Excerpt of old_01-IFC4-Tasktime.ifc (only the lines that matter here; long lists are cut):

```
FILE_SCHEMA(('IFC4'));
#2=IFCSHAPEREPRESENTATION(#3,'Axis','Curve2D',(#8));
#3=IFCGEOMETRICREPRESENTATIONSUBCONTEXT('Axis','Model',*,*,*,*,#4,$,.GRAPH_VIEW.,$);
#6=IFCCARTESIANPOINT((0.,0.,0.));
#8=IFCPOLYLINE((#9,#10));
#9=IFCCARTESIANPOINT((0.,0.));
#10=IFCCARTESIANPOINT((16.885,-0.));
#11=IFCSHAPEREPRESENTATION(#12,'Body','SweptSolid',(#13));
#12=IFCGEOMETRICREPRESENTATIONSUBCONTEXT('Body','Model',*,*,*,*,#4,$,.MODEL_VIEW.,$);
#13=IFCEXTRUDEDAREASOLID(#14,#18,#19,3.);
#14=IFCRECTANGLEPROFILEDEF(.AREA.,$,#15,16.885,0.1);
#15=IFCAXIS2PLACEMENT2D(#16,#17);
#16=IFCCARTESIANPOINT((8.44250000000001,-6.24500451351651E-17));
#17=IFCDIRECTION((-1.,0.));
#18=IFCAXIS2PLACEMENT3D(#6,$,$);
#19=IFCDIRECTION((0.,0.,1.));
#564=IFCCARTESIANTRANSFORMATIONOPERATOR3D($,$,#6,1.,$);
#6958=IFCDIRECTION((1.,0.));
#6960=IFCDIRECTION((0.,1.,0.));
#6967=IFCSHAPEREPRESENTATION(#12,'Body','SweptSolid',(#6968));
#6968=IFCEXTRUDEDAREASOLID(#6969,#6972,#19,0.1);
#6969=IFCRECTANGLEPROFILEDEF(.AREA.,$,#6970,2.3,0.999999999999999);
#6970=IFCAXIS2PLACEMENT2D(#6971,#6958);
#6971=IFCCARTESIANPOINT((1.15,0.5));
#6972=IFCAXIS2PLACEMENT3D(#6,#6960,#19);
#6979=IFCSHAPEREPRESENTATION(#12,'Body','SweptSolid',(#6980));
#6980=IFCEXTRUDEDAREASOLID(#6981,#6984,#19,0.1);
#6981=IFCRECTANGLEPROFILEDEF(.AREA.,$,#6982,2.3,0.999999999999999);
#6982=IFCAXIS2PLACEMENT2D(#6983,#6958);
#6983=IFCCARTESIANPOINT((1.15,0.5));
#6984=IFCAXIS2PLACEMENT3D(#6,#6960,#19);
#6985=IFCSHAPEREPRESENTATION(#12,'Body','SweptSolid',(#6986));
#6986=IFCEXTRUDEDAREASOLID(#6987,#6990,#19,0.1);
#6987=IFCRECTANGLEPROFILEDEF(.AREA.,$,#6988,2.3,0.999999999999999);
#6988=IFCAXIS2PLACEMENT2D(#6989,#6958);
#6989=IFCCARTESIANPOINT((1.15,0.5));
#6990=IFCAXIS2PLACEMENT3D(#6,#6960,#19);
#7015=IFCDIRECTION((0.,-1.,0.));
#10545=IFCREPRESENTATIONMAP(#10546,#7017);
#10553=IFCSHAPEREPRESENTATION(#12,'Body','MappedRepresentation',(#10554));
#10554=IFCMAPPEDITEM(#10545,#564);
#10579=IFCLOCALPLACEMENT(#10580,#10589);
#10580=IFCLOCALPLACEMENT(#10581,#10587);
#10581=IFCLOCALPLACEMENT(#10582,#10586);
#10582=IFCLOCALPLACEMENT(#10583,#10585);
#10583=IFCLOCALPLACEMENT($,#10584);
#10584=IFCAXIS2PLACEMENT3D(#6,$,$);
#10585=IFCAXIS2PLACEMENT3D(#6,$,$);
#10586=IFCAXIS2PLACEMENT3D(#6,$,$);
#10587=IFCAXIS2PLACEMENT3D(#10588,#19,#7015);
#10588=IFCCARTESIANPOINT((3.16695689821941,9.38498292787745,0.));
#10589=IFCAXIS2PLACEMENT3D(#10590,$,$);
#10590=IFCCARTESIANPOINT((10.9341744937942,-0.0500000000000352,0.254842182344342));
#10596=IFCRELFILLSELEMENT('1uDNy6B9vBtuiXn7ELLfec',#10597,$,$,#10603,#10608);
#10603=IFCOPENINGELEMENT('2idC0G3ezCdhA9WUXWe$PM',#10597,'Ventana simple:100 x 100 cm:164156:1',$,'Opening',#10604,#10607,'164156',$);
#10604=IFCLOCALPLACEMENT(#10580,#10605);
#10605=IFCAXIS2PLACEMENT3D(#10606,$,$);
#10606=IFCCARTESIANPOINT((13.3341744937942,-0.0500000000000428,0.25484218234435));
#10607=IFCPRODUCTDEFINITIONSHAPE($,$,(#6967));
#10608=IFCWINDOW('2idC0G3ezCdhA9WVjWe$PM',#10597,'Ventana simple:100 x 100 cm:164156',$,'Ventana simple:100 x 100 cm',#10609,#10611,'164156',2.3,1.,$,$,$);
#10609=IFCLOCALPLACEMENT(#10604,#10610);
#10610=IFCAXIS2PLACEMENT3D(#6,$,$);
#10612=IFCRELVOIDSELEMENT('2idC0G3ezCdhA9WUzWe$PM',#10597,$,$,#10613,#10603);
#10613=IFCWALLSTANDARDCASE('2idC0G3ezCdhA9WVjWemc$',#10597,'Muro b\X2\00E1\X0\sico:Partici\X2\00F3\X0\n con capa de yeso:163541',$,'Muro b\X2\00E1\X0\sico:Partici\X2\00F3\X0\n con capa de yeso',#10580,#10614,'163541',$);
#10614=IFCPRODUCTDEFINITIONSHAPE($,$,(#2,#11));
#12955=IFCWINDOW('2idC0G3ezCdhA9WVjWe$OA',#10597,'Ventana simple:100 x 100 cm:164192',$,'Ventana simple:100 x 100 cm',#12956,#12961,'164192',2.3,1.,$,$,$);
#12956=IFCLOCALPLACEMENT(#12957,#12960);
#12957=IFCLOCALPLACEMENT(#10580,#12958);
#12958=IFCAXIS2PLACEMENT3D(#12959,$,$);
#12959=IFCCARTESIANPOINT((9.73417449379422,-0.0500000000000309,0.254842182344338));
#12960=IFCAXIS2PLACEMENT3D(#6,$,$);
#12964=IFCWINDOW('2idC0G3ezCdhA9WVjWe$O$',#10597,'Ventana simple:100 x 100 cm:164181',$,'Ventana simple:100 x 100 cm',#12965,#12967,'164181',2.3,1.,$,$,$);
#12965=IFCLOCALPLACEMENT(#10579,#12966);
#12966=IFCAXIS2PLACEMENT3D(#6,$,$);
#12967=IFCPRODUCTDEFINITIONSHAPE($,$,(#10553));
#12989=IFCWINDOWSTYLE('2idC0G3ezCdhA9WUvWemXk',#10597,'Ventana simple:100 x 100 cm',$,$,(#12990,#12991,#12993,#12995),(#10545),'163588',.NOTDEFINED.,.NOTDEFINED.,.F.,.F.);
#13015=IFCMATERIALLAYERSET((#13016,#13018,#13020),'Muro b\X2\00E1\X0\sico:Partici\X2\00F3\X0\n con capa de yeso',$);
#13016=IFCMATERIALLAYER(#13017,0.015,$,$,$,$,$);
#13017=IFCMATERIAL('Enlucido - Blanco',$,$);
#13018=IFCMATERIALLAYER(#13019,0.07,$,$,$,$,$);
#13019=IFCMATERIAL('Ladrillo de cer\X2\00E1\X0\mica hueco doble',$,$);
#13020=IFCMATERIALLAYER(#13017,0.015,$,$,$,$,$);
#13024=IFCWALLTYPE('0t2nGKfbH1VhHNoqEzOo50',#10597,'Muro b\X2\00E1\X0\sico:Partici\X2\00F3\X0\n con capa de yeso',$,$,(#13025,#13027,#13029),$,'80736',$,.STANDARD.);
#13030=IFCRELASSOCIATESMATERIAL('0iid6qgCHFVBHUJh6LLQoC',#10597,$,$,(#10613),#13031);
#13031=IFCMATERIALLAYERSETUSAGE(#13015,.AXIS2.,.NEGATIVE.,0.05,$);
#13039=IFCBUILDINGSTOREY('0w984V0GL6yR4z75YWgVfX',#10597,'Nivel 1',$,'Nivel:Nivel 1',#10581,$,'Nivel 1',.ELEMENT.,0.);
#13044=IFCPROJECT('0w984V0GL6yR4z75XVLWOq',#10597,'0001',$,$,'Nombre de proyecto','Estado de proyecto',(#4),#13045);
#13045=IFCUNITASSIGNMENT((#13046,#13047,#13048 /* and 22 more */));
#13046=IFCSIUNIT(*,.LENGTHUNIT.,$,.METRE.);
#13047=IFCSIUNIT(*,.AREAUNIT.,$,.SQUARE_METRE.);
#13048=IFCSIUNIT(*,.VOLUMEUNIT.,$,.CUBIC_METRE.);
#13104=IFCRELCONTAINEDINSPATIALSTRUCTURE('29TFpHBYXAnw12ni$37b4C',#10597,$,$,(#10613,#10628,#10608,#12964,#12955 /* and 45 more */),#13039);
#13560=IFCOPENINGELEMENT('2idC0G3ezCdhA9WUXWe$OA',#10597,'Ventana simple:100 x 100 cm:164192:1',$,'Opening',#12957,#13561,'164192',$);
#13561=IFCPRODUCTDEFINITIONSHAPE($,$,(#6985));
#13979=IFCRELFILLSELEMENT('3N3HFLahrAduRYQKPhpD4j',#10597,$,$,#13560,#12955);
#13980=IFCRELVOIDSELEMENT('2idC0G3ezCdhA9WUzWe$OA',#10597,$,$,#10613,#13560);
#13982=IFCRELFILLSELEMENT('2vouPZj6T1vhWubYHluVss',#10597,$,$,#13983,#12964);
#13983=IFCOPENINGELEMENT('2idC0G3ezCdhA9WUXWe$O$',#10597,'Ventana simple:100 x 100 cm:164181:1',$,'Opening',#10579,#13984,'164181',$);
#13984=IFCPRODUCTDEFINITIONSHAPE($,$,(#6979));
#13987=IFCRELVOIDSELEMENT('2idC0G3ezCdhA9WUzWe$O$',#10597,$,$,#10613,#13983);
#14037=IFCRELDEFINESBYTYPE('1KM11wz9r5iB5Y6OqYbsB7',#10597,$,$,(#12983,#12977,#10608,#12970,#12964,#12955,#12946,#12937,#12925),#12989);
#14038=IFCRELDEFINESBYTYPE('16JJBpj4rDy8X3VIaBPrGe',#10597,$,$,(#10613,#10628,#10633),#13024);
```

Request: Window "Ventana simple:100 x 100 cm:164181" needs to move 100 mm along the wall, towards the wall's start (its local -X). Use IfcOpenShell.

```python
import ifcopenshell
import ifcopenshell.api.geometry
import ifcopenshell.util.placement

model = ifcopenshell.open("old_01-IFC4-Tasktime.ifc")

window = model.by_guid("2idC0G3ezCdhA9WVjWe$O$")
opening = window.FillsVoids[0].RelatingOpeningElement
wall = opening.VoidsElements[0].RelatingBuildingElement

wall_matrix = ifcopenshell.util.placement.get_local_placement(wall.ObjectPlacement)
shift = wall_matrix[:3, 0] * -0.1
before = ifcopenshell.util.placement.get_local_placement(window.ObjectPlacement)[:3, 3].copy()

# The window is placed relative to its opening, so it follows when the opening moves.
matrix = ifcopenshell.util.placement.get_local_placement(opening.ObjectPlacement)
matrix[:3, 3] += shift
ifcopenshell.api.geometry.edit_object_placement(
    model, product=opening, matrix=matrix, is_si=False, should_transform_children=True
)

after = ifcopenshell.util.placement.get_local_placement(window.ObjectPlacement)[:3, 3]
print("window moved by", (after - before).round(3) + 0.0)

model.write("old_01-IFC4-Tasktime-out.ifc")
```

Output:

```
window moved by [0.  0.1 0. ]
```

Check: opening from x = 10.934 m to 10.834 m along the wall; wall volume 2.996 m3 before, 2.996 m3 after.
